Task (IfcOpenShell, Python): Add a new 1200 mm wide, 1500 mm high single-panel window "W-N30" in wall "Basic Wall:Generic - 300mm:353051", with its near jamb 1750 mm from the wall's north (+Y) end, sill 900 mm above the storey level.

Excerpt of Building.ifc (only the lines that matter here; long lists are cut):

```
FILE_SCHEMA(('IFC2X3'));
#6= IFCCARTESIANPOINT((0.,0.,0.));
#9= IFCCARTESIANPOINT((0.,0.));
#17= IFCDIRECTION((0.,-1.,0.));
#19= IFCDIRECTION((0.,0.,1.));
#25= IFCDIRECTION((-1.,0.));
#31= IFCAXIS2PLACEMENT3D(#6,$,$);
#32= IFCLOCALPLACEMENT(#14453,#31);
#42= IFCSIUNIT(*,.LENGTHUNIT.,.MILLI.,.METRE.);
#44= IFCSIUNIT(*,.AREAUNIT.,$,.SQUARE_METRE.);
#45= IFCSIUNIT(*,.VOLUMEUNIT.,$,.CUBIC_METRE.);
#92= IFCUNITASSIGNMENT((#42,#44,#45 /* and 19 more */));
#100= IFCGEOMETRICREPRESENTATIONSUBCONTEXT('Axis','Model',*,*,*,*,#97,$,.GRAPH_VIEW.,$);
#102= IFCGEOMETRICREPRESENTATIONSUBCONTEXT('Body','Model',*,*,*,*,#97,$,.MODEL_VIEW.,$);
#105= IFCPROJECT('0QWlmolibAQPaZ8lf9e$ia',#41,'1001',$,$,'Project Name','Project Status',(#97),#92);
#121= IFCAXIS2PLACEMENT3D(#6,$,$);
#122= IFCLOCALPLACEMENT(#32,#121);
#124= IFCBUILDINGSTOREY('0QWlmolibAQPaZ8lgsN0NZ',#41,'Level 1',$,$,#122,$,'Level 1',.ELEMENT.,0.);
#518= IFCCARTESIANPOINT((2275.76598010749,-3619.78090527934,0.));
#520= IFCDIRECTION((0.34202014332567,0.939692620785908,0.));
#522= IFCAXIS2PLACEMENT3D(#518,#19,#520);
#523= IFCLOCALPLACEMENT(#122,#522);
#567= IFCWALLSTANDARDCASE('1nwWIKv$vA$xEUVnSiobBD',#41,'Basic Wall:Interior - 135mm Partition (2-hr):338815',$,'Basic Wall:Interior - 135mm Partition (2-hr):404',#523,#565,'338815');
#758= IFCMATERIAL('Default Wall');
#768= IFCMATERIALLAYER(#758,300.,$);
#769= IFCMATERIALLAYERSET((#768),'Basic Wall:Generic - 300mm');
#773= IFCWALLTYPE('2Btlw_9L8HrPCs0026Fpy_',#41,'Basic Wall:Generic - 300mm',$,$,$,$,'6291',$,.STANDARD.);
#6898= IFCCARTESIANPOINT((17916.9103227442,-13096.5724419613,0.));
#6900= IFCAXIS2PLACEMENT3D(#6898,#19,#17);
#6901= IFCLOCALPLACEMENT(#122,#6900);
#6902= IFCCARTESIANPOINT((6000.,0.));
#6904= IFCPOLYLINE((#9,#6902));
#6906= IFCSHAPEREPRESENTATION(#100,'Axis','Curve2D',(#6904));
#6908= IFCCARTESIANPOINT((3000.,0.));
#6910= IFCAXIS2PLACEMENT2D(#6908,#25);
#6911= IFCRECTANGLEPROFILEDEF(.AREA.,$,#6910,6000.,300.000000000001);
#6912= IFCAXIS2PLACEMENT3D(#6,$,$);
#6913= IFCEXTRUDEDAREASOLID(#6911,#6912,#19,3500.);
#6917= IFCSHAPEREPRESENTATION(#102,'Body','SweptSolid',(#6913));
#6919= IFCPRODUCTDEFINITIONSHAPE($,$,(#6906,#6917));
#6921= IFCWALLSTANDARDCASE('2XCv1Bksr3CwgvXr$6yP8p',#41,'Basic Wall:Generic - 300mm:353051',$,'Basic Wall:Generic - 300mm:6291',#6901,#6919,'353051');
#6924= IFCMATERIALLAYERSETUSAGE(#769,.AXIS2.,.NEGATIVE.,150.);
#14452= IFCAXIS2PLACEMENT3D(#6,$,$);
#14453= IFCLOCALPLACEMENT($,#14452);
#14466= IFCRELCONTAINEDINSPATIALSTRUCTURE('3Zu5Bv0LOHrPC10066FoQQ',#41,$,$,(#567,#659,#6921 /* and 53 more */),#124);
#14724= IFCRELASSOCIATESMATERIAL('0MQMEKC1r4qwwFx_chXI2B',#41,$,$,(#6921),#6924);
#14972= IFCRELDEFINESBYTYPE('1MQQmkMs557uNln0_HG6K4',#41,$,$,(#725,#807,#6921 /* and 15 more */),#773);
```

```python
import numpy as np
import ifcopenshell
import ifcopenshell.api.feature
import ifcopenshell.api.geometry
import ifcopenshell.api.root
import ifcopenshell.api.spatial
import ifcopenshell.api.type
import ifcopenshell.geom
import ifcopenshell.util.element
import ifcopenshell.util.placement
import ifcopenshell.util.representation
import ifcopenshell.util.shape
import ifcopenshell.util.unit

model = ifcopenshell.open("Building.ifc")
unit_scale = ifcopenshell.util.unit.calculate_unit_scale(model)
settings = ifcopenshell.geom.settings()


def volume(element):
    """Net volume in cubic metres, openings subtracted."""
    shape = ifcopenshell.geom.create_shape(settings, element)
    return ifcopenshell.util.shape.get_volume(shape.geometry)


wall = model.by_guid("2XCv1Bksr3CwgvXr$6yP8p")
storey = ifcopenshell.util.element.get_container(wall, ifc_class="IfcBuildingStorey")
context = ifcopenshell.util.representation.get_context(model, "Model", "Body", "MODEL_VIEW")
before = volume(wall)

width, height, from_end, sill = 1.2, 1.5, 1.75, 0.9  # metres

# The wall runs along its own X axis, and the end named is its -X end.
wall_shape = ifcopenshell.geom.create_shape(settings, wall)
x, y, z = ifcopenshell.util.shape.get_vertices(wall_shape.geometry).T
start = x.min() + from_end
face, thickness = float(y.min()), float(y.max() - y.min())
wall_matrix = ifcopenshell.util.placement.get_local_placement(wall.ObjectPlacement)
level = ifcopenshell.util.placement.get_local_placement(storey.ObjectPlacement)[2, 3]


def in_wall(x, y):
    """Placement at x, y metres in the wall's axes, at sill height."""
    matrix = wall_matrix.copy()
    matrix[:, 3] = wall_matrix @ np.array([x / unit_scale, y / unit_scale, 0.0, 1.0])
    matrix[2, 3] = level + sill / unit_scale
    return matrix


# Opening: a box that overshoots both wall faces by 50 mm.
opening = ifcopenshell.api.root.create_entity(model, ifc_class="IfcOpeningElement")
box = ifcopenshell.api.geometry.add_wall_representation(
    model, context=context, length=width, height=height, thickness=thickness + 0.1
)
ifcopenshell.api.geometry.assign_representation(model, product=opening, representation=box)
ifcopenshell.api.geometry.edit_object_placement(model, product=opening, matrix=in_wall(start, face - 0.05), is_si=False)
ifcopenshell.api.feature.add_feature(model, feature=opening, element=wall)

window = ifcopenshell.api.root.create_entity(model, ifc_class="IfcWindow", name="W-N30")
window.OverallWidth, window.OverallHeight = width / unit_scale, height / unit_scale
body = ifcopenshell.api.geometry.add_window_representation(
    model,
    context=context,
    overall_width=window.OverallWidth,
    overall_height=window.OverallHeight,
    partition_type="SINGLE_PANEL",
)
ifcopenshell.api.geometry.assign_representation(model, product=window, representation=body)
ifcopenshell.api.spatial.assign_container(model, products=[window], relating_structure=storey)
fills = ifcopenshell.api.feature.add_filling(model, opening=opening, element=window)
fills.OwnerHistory = window.OwnerHistory  # required in IFC2X3

# IFC2X3 keeps the operation on the window style.
style = ifcopenshell.api.root.create_entity(model, ifc_class="IfcWindowStyle", name="W-N30")
style.OperationType, style.ConstructionType = "SINGLE_PANEL", "NOTDEFINED"
style.ParameterTakesPrecedence = style.Sizeable = False
ifcopenshell.api.type.assign_type(model, related_objects=[window], relating_type=style)

# Centre the window in the wall's thickness.
ifcopenshell.api.geometry.edit_object_placement(model, product=window, matrix=in_wall(start, face), is_si=False)
window_shape = ifcopenshell.geom.create_shape(settings, window)
depth = ifcopenshell.util.shape.get_vertices(window_shape.geometry)[:, 1]
offset = face + thickness / 2 - (depth.min() + depth.max()) / 2
ifcopenshell.api.geometry.edit_object_placement(model, product=window, matrix=in_wall(start, offset), is_si=False)

after = volume(wall)

print(f"wall volume {before:.3f} -> {after:.3f} m3")

model.write("Building-out.ifc")
```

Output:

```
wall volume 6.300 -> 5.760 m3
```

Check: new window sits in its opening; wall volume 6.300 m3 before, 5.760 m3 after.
